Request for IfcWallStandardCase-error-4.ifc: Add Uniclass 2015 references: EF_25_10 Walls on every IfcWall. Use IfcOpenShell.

First a look at what the model holds.

```python
import ifcopenshell

model = ifcopenshell.open("IfcWallStandardCase-error-4.ifc")
print(model.schema)
print("classifications:", [c.Name for c in model.by_type("IfcClassification")])
for ifc_class in ("IfcDoor", "IfcRoof", "IfcStair", "IfcWall", "IfcWindow"):
    print(ifc_class, len(model.by_type(ifc_class)))
```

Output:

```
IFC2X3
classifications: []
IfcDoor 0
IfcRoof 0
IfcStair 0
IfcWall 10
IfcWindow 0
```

```python
import ifcopenshell
import ifcopenshell.api.classification

model = ifcopenshell.open("IfcWallStandardCase-error-4.ifc")

# IFC2X3 requires Source and Edition and has no link from the project to the system.
system = model.create_entity("IfcClassification", Source="NBS", Edition="2015", Name="Uniclass 2015")

codes = {
    "IfcWall": ("EF_25_10", "Walls"),
}
for ifc_class, (code, name) in codes.items():
    products = model.by_type(ifc_class)
    ifcopenshell.api.classification.add_reference(
        model, products=products, classification=system, identification=code, name=name
    )
    print(code, len(products))

model.write("IfcWallStandardCase-error-4-out.ifc")
```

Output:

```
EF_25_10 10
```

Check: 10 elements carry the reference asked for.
